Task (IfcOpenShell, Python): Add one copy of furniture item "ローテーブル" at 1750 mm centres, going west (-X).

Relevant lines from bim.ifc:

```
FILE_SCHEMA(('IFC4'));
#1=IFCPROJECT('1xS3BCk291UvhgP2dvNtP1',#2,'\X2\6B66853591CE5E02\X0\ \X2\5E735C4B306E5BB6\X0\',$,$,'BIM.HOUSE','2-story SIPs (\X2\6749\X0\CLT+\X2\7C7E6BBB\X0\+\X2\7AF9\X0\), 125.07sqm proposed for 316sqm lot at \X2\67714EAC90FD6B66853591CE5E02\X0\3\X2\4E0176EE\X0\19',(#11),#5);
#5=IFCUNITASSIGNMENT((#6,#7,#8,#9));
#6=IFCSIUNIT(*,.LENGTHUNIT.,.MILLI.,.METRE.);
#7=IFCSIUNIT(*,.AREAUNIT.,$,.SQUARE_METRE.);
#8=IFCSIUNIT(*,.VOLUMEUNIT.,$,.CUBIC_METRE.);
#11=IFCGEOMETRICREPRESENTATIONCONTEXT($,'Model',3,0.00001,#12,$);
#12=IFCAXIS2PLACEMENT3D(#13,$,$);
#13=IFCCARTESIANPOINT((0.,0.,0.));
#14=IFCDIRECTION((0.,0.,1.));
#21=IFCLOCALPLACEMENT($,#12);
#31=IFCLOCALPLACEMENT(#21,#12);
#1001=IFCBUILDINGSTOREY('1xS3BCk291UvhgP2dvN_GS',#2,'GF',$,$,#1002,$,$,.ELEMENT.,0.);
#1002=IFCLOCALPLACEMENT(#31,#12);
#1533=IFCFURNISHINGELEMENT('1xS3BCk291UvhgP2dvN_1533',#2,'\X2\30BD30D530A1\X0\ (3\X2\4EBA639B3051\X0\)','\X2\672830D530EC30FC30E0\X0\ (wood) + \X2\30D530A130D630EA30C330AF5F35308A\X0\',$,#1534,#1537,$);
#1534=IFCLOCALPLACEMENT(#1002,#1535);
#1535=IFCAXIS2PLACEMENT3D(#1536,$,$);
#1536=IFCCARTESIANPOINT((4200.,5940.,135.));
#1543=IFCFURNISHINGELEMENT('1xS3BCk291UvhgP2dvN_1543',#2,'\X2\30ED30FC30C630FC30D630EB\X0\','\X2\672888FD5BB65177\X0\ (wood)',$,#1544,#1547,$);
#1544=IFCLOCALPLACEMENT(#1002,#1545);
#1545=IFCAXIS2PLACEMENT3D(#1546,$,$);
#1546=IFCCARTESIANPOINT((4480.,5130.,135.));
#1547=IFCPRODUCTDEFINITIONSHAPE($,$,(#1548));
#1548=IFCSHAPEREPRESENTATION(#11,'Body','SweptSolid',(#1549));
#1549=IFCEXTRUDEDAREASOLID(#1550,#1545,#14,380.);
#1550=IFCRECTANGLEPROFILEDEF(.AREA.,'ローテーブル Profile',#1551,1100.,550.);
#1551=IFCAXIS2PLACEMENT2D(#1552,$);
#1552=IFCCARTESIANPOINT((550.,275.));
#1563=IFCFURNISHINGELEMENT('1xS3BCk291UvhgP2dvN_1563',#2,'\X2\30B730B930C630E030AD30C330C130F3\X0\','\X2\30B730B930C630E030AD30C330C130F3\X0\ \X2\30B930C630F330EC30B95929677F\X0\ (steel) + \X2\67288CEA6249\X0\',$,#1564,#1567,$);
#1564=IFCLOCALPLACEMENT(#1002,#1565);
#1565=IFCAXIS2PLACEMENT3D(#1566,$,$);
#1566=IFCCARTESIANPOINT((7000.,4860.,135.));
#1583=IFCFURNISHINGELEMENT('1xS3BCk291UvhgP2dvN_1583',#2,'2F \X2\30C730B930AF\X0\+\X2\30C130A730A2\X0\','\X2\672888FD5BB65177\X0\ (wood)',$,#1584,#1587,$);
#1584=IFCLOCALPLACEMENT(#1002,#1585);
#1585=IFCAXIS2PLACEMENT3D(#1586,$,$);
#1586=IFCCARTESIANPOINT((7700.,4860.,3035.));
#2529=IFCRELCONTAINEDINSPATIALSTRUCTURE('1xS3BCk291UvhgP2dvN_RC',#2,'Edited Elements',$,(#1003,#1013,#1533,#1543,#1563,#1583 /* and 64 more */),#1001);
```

```python
import numpy as np
import ifcopenshell
import ifcopenshell.api.geometry
import ifcopenshell.api.root
import ifcopenshell.util.element
import ifcopenshell.util.placement

model = ifcopenshell.open("bim.ifc")


def reuse_history(source, copy):
    """copy_class also copies each property set's owner history, people and application; keep the originals."""
    for rel in copy.IsDefinedBy:
        if rel.is_a("IfcRelDefinesByProperties") and (history := rel.RelatingPropertyDefinition.OwnerHistory):
            rel.RelatingPropertyDefinition.OwnerHistory = source.OwnerHistory
            ifcopenshell.util.element.remove_deep2(model, history)


source = model.by_guid("1xS3BCk291UvhgP2dvN_1543")
base = ifcopenshell.util.placement.get_local_placement(source.ObjectPlacement)
step = np.array([-1.0, 0.0, 0.0]) * 1750.0

for i in range(1, 2):
    copy = ifcopenshell.api.root.copy_class(model, product=source)
    copy.Representation = ifcopenshell.util.element.copy_deep(
        model, source.Representation, exclude=["IfcGeometricRepresentationContext", "IfcRepresentationMap"]
    )
    reuse_history(source, copy)
    matrix = base.copy()
    matrix[:3, 3] += i * step
    print("added at", matrix[:3, 3].round(3) + 0.0)
    ifcopenshell.api.geometry.edit_object_placement(model, product=copy, matrix=matrix, is_si=False)

model.write("bim_updated.ifc")
```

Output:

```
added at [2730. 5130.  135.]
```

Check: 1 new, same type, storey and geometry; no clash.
